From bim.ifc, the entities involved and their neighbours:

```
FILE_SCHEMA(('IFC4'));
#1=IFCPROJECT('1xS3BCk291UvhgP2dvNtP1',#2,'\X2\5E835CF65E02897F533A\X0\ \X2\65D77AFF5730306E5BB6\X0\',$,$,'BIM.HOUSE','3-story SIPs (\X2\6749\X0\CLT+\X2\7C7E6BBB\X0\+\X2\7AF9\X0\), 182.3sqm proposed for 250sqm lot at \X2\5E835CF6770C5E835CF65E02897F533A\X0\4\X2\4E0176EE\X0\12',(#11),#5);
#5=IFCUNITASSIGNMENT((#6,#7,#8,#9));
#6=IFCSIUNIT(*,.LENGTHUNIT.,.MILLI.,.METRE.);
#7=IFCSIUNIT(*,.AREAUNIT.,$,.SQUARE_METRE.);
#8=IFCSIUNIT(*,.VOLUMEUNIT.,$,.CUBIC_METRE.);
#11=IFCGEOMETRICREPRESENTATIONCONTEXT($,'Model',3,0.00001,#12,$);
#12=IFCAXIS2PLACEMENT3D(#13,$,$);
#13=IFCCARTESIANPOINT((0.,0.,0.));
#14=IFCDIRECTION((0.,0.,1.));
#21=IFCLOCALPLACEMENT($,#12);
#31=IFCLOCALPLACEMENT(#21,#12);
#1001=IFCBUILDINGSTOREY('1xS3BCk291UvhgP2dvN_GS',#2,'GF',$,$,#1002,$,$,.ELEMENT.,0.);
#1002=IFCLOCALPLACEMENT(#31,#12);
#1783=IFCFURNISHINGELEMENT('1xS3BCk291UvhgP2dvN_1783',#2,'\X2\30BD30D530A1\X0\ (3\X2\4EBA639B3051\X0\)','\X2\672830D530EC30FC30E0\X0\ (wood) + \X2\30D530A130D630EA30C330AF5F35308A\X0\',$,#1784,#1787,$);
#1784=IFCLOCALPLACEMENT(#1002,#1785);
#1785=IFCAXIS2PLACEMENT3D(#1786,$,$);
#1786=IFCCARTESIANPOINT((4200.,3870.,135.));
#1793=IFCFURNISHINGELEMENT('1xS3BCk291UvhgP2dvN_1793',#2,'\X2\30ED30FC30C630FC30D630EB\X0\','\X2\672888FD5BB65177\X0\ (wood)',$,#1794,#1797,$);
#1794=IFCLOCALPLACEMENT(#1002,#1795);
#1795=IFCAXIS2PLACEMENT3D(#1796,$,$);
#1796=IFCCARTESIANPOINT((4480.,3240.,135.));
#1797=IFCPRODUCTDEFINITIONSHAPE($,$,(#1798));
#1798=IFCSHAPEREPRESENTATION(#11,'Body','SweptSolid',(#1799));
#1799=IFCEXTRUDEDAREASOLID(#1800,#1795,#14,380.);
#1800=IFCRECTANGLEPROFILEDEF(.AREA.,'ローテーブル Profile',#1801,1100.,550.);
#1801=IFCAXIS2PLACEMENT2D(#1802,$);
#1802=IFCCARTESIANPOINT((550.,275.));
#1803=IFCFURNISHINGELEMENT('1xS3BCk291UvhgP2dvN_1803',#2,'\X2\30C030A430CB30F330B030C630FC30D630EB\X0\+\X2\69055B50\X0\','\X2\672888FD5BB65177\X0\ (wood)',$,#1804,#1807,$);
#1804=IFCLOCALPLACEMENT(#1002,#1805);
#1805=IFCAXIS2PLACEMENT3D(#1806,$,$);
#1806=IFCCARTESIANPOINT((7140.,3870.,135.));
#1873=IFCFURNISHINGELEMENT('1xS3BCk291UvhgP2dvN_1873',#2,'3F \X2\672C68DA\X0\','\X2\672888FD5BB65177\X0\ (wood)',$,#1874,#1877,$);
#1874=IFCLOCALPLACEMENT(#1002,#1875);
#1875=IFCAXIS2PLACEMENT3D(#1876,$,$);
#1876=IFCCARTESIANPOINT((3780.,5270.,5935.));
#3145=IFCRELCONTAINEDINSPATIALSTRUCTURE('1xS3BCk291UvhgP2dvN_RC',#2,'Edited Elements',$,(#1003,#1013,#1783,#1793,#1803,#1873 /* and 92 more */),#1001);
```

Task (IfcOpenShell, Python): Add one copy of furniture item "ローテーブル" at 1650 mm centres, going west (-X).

```python
import numpy as np
import ifcopenshell
import ifcopenshell.api.geometry
import ifcopenshell.api.root
import ifcopenshell.util.element
import ifcopenshell.util.placement

model = ifcopenshell.open("bim.ifc")


def reuse_history(source, copy):
    """copy_class also copies each property set's owner history, people and application; keep the originals."""
    for rel in copy.IsDefinedBy:
        if rel.is_a("IfcRelDefinesByProperties") and (history := rel.RelatingPropertyDefinition.OwnerHistory):
            rel.RelatingPropertyDefinition.OwnerHistory = source.OwnerHistory
            ifcopenshell.util.element.remove_deep2(model, history)


source = model.by_guid("1xS3BCk291UvhgP2dvN_1793")
base = ifcopenshell.util.placement.get_local_placement(source.ObjectPlacement)
step = np.array([-1.0, 0.0, 0.0]) * 1650.0

for i in range(1, 2):
    copy = ifcopenshell.api.root.copy_class(model, product=source)
    copy.Representation = ifcopenshell.util.element.copy_deep(
        model, source.Representation, exclude=["IfcGeometricRepresentationContext", "IfcRepresentationMap"]
    )
    reuse_history(source, copy)
    matrix = base.copy()
    matrix[:3, 3] += i * step
    print("added at", matrix[:3, 3].round(3) + 0.0)
    ifcopenshell.api.geometry.edit_object_placement(model, product=copy, matrix=matrix, is_si=False)

model.write("bim_edited.ifc")
```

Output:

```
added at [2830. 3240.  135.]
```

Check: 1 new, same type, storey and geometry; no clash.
